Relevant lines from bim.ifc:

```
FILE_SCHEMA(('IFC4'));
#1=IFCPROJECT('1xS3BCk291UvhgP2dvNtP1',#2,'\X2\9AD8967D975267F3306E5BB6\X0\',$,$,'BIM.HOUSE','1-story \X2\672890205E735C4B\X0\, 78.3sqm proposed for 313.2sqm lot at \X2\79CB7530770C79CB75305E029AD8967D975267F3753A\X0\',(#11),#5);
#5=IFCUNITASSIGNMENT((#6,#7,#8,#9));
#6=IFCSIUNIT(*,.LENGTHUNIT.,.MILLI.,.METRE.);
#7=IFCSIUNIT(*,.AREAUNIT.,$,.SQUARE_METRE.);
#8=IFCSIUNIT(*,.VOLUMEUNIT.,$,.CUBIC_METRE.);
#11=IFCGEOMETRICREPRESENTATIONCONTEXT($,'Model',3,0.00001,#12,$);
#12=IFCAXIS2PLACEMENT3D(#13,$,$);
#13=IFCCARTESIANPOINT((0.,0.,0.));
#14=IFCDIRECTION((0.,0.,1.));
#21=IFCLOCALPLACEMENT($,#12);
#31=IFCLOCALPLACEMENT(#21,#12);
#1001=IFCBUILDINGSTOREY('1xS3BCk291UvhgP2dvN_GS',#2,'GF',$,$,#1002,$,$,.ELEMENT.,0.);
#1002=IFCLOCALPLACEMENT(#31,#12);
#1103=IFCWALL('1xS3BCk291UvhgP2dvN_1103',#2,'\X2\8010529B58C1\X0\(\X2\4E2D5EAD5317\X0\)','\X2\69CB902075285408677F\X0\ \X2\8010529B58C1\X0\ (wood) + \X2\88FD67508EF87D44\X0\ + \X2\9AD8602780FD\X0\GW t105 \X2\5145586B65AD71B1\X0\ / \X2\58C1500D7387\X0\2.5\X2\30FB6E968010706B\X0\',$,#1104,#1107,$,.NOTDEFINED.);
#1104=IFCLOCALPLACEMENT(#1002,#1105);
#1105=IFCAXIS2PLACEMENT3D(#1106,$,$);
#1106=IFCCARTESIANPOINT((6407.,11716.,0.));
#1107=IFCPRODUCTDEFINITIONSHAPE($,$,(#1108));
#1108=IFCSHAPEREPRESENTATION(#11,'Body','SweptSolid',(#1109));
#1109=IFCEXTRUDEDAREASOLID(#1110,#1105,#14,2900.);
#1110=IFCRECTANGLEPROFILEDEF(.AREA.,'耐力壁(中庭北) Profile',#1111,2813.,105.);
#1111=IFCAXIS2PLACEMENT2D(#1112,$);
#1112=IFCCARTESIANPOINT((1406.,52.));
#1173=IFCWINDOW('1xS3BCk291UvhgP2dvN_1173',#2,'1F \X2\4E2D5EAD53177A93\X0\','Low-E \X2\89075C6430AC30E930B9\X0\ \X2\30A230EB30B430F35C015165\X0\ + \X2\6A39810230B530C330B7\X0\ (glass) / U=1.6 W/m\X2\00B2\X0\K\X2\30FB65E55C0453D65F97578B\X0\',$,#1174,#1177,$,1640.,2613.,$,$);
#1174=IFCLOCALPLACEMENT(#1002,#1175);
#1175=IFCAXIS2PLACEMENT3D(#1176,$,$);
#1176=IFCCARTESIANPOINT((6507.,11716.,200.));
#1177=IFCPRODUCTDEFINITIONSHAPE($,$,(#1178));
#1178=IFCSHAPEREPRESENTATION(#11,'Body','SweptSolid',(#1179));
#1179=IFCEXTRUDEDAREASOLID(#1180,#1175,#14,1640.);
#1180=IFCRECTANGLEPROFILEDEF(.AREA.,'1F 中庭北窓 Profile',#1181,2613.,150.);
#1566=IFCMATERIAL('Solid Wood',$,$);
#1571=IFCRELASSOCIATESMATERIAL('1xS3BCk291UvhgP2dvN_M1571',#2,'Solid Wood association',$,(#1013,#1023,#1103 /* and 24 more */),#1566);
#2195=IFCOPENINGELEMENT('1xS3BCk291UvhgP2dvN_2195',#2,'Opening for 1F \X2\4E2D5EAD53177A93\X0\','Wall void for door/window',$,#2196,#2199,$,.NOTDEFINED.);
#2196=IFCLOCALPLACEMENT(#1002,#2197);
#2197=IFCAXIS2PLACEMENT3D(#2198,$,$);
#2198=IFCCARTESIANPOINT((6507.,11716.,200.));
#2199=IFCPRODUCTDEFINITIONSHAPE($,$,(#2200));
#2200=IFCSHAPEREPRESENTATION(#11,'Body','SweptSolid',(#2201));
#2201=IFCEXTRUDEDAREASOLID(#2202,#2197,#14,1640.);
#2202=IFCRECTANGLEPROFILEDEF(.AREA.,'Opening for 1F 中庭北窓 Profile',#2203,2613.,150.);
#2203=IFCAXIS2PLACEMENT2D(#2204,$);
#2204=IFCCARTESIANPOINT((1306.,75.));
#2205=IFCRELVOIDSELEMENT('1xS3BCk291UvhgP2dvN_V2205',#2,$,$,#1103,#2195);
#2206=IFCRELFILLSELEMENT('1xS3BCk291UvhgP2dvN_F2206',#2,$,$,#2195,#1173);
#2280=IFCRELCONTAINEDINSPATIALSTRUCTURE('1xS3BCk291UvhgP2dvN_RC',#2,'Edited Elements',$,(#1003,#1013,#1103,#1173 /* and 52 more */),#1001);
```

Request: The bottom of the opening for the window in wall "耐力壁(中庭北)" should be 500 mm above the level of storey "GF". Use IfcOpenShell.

```python
import numpy as np
import ifcopenshell
import ifcopenshell.api.geometry
import ifcopenshell.geom
import ifcopenshell.util.element
import ifcopenshell.util.placement
import ifcopenshell.util.shape
import ifcopenshell.util.unit

model = ifcopenshell.open("bim.ifc")
unit_scale = ifcopenshell.util.unit.calculate_unit_scale(model)

window = model.by_guid("1xS3BCk291UvhgP2dvN_1173")
opening = window.FillsVoids[0].RelatingOpeningElement
storey = ifcopenshell.util.element.get_container(window, ifc_class="IfcBuildingStorey")
level = ifcopenshell.util.placement.get_local_placement(storey.ObjectPlacement)[2, 3]

# The opening's origin need not be at the sill, so measure its lowest point.
shape = ifcopenshell.geom.create_shape(ifcopenshell.geom.settings(), opening)
bottom = ifcopenshell.util.shape.get_shape_bottom_elevation(shape, shape.geometry) / unit_scale
dz = level + 0.5 / unit_scale - bottom

shift = np.array([0.0, 0.0, dz])
# The window is not placed relative to its opening, so move both.
for product in (opening, window):
    matrix = ifcopenshell.util.placement.get_local_placement(product.ObjectPlacement)
    matrix[:3, 3] += shift
    ifcopenshell.api.geometry.edit_object_placement(model, product=product, matrix=matrix, is_si=False)

print(f"moved by {dz * unit_scale:+.3f} m")

model.write("bim_edited.ifc")
```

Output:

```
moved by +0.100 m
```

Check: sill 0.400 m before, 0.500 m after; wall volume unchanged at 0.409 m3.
